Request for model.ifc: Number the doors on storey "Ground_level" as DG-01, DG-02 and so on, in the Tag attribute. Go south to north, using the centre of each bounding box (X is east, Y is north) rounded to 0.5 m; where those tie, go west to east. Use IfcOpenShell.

First a look at what the model holds.

```python
import ifcopenshell
import ifcopenshell.util.element
import ifcopenshell.util.placement

model = ifcopenshell.open("model.ifc")
print(model.schema)
storey = next(s for s in model.by_type("IfcBuildingStorey") if s.Name == "Ground_level")
doors = [e for e in ifcopenshell.util.element.get_decomposition(storey) if e.is_a("IfcDoor")]
for e in sorted(doors, key=lambda e: e.id()):
    origin = ifcopenshell.util.placement.get_local_placement(e.ObjectPlacement)[:3, 3]
    print(e.id(), e.Tag, e.Name, origin.round(2) + 0.0, sep=" | ")
```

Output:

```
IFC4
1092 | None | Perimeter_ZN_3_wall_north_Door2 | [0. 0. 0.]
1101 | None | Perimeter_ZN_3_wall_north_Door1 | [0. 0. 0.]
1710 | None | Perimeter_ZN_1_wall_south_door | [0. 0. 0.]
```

```python
import ifcopenshell
import ifcopenshell.geom
import ifcopenshell.util.element
import ifcopenshell.util.shape

model = ifcopenshell.open("model.ifc")
settings = ifcopenshell.geom.settings()
settings.set("use-world-coords", True)


def centre(element):
    shape = ifcopenshell.geom.create_shape(settings, element)
    return ifcopenshell.util.shape.get_bbox_centroid(shape.geometry)


storey = next(s for s in model.by_type("IfcBuildingStorey") if s.Name == "Ground_level")
doors = [e for e in ifcopenshell.util.element.get_decomposition(storey) if e.is_a("IfcDoor")]

# Insertion points can sit at a corner or the storey origin, so sort by the geometry (in metres).
centres = {e: centre(e) for e in doors}
doors.sort(key=lambda e: (round(centres[e][1] / 0.5), centres[e][0]))

for i, e in enumerate(doors, start=1):
    number = f"DG-{i:02d}"
    e.Tag = number
    print(e.id(), number)

model.write("model_edited.ifc")
```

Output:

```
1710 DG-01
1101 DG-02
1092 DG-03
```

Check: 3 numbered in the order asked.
